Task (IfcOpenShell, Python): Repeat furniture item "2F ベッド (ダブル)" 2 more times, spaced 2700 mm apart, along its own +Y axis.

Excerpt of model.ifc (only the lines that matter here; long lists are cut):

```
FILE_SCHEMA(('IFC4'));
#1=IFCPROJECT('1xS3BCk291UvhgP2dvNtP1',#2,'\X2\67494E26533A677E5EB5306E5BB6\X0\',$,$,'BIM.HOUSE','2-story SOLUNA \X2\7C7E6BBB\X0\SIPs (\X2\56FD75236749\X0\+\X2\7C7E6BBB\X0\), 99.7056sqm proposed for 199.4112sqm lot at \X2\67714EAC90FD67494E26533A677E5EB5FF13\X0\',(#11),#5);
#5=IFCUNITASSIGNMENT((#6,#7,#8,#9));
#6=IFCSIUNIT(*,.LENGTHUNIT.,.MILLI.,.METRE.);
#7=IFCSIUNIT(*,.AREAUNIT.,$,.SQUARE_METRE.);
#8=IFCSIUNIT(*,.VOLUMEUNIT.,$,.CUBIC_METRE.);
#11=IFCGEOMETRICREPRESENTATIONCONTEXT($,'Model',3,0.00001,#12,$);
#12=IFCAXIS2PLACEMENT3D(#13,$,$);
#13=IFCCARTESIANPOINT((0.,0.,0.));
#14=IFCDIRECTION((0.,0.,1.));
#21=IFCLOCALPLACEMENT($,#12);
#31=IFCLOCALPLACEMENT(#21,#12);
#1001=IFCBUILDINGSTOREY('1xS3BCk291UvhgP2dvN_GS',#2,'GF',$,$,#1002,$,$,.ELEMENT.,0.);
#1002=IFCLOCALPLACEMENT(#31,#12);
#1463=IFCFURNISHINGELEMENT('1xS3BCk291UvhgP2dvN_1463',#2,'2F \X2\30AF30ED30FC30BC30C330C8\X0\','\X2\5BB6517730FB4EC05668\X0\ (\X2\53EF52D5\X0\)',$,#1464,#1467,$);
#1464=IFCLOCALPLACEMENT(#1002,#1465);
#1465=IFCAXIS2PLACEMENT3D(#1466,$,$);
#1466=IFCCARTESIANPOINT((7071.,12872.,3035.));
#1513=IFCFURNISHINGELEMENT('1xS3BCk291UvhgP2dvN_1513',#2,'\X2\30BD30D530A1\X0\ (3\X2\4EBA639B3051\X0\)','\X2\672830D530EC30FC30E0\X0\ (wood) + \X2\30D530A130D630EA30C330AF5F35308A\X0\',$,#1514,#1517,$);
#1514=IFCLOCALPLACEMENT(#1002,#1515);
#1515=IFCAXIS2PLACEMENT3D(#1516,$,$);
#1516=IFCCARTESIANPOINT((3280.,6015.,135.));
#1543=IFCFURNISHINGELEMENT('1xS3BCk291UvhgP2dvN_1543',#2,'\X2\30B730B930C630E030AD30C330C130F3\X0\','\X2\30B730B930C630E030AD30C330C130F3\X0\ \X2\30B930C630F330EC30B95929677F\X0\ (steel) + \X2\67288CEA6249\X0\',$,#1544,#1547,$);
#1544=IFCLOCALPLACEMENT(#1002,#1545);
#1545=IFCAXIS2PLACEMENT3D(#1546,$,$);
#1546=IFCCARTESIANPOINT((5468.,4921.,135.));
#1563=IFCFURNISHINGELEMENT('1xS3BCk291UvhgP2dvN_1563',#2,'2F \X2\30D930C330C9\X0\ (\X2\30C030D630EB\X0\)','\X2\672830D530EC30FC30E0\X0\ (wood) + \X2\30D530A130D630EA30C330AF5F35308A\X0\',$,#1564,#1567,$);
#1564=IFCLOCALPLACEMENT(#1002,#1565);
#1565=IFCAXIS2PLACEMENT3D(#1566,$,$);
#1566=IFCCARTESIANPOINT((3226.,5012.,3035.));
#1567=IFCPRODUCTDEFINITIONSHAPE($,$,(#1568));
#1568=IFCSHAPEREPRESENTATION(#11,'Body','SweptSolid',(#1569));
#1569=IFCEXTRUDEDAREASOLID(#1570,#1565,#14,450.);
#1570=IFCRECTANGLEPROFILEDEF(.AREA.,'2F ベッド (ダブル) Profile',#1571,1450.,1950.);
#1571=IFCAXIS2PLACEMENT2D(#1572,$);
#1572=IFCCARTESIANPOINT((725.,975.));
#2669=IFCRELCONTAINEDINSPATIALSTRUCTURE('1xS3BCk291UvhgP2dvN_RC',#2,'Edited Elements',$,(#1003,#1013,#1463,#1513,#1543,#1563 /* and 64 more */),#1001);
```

```python
import ifcopenshell
import ifcopenshell.api.geometry
import ifcopenshell.api.root
import ifcopenshell.util.element
import ifcopenshell.util.placement

model = ifcopenshell.open("model.ifc")


def reuse_history(source, copy):
    """copy_class also copies each property set's owner history, people and application; keep the originals."""
    for rel in copy.IsDefinedBy:
        if rel.is_a("IfcRelDefinesByProperties") and (history := rel.RelatingPropertyDefinition.OwnerHistory):
            rel.RelatingPropertyDefinition.OwnerHistory = source.OwnerHistory
            ifcopenshell.util.element.remove_deep2(model, history)


source = model.by_guid("1xS3BCk291UvhgP2dvN_1563")
base = ifcopenshell.util.placement.get_local_placement(source.ObjectPlacement)
step = base[:3, 1] * 2700.0

for i in range(1, 3):
    copy = ifcopenshell.api.root.copy_class(model, product=source)
    copy.Representation = ifcopenshell.util.element.copy_deep(
        model, source.Representation, exclude=["IfcGeometricRepresentationContext", "IfcRepresentationMap"]
    )
    reuse_history(source, copy)
    matrix = base.copy()
    matrix[:3, 3] += i * step
    print("added at", matrix[:3, 3].round(3) + 0.0)
    ifcopenshell.api.geometry.edit_object_placement(model, product=copy, matrix=matrix, is_si=False)

model.write("model_updated.ifc")
```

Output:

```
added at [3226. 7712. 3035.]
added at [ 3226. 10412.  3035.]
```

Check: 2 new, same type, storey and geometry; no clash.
